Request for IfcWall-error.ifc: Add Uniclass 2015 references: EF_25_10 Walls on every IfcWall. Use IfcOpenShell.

First a look at what the model holds.

```python
import ifcopenshell

model = ifcopenshell.open("IfcWall-error.ifc")
print(model.schema)
print("classifications:", [c.Name for c in model.by_type("IfcClassification")])
for ifc_class in ("IfcDoor", "IfcRoof", "IfcStair", "IfcWall", "IfcWindow"):
    print(ifc_class, len(model.by_type(ifc_class)))
```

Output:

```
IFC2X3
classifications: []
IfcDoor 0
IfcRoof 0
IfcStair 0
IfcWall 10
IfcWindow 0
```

```python
import ifcopenshell
import ifcopenshell.api.classification

model = ifcopenshell.open("IfcWall-error.ifc")

# IFC2X3 requires Source and Edition and has no link from the project to the system.
system = model.create_entity("IfcClassification", Source="NBS", Edition="2015", Name="Uniclass 2015")

codes = {
    "IfcWall": ("EF_25_10", "Walls"),
}
for ifc_class, (code, name) in codes.items():
    products = model.by_type(ifc_class)
    ifcopenshell.api.classification.add_reference(
        model, products=products, classification=system, identification=code, name=name
    )
    print(code, len(products))

model.write("IfcWall-error_rev.ifc")
```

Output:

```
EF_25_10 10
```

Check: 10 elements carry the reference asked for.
